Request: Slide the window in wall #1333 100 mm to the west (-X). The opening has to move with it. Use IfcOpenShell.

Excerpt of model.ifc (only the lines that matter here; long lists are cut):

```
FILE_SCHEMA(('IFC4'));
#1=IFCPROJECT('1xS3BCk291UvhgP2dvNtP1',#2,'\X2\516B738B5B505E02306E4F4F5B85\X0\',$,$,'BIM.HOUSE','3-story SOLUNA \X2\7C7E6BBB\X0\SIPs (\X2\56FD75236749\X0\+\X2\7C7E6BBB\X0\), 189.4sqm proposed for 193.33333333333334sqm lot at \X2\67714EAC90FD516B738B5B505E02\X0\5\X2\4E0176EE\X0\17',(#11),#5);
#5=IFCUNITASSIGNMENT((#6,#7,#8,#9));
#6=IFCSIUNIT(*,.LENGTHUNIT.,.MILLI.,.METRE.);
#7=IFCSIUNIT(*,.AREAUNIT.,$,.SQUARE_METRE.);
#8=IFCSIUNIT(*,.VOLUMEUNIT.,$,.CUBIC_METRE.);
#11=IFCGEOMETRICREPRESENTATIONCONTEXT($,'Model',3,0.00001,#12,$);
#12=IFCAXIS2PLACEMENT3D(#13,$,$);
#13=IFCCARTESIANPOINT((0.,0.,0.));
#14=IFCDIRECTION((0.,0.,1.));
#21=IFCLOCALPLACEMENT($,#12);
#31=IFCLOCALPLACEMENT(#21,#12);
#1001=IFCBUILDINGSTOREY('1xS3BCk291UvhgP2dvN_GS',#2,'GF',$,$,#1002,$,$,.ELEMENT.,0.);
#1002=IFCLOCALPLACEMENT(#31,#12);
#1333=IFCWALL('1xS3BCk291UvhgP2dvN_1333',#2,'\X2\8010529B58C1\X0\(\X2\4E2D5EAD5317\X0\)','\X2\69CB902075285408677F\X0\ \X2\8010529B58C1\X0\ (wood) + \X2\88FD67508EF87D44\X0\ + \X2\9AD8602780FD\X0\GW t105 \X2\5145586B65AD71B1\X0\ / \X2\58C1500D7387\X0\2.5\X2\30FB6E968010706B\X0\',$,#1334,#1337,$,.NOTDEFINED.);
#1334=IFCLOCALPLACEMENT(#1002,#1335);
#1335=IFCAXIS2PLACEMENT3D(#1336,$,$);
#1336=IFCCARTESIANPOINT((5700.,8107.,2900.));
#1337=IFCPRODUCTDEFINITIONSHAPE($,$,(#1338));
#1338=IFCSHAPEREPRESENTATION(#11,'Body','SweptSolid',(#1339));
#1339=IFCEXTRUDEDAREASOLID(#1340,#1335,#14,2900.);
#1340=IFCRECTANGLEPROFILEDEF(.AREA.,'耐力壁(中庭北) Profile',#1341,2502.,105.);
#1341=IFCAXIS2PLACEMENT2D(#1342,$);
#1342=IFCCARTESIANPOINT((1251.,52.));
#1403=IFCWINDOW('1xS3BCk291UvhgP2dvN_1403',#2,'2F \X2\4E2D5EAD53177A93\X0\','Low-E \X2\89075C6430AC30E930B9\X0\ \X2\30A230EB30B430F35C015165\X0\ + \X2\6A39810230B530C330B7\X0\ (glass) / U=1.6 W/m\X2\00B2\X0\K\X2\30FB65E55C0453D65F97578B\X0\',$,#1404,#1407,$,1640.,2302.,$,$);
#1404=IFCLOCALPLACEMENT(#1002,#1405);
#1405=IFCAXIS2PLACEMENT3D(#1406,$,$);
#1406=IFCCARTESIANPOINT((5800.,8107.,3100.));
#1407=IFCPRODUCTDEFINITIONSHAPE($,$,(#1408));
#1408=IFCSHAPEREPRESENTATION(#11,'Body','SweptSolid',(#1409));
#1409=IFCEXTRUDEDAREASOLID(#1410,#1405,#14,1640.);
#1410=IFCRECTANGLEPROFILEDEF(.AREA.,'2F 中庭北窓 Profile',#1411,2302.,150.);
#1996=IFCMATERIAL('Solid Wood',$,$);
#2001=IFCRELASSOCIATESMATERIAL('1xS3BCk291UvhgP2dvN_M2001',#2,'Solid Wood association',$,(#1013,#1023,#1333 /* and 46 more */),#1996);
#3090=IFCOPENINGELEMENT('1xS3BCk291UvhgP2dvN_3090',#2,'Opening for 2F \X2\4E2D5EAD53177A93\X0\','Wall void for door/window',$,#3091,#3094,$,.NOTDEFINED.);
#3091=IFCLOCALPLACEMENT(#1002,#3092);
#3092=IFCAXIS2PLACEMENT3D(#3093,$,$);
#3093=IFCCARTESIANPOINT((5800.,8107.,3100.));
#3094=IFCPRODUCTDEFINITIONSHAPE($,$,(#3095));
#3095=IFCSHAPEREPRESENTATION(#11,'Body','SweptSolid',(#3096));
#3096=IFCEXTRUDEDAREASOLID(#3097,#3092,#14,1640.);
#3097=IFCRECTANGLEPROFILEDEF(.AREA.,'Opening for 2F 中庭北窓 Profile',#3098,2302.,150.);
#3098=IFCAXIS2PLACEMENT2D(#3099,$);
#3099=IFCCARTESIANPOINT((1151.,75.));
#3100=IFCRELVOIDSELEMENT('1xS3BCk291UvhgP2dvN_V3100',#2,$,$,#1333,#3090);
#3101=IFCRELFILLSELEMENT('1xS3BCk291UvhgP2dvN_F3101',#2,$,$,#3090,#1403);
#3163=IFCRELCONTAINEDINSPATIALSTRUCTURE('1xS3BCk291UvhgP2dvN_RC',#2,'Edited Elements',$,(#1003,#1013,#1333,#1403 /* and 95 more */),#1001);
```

```python
import ifcopenshell
import ifcopenshell.api.geometry
import ifcopenshell.util.placement
import ifcopenshell.util.unit

model = ifcopenshell.open("model.ifc")
unit_scale = ifcopenshell.util.unit.calculate_unit_scale(model)

window = model.by_guid("1xS3BCk291UvhgP2dvN_1403")
opening = window.FillsVoids[0].RelatingOpeningElement
wall = opening.VoidsElements[0].RelatingBuildingElement

wall_matrix = ifcopenshell.util.placement.get_local_placement(wall.ObjectPlacement)
shift = wall_matrix[:3, 0] * -0.1 / unit_scale
before = ifcopenshell.util.placement.get_local_placement(window.ObjectPlacement)[:3, 3].copy()

# The window is not placed relative to its opening, so move both.
for product in (opening, window):
    matrix = ifcopenshell.util.placement.get_local_placement(product.ObjectPlacement)
    matrix[:3, 3] += shift
    ifcopenshell.api.geometry.edit_object_placement(model, product=product, matrix=matrix, is_si=False)

after = ifcopenshell.util.placement.get_local_placement(window.ObjectPlacement)[:3, 3]
print("window moved by", (after - before).round(3) + 0.0)

model.write("model_rev.ifc")
```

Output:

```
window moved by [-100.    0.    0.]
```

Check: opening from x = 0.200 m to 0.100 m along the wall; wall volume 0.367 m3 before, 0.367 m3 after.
